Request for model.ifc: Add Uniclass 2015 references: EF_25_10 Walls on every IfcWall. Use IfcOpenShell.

First a look at what the model holds.

```python
import ifcopenshell

model = ifcopenshell.open("model.ifc")
print(model.schema)
print("classifications:", [c.Name for c in model.by_type("IfcClassification")])
for ifc_class in ("IfcDoor", "IfcRoof", "IfcStair", "IfcWall", "IfcWindow"):
    print(ifc_class, len(model.by_type(ifc_class)))
```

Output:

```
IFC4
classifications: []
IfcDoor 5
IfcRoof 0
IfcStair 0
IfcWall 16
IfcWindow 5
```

```python
import ifcopenshell
import ifcopenshell.api.classification

model = ifcopenshell.open("model.ifc")

system = ifcopenshell.api.classification.add_classification(model, classification="Uniclass 2015")

codes = {
    "IfcWall": ("EF_25_10", "Walls"),
}
for ifc_class, (code, name) in codes.items():
    products = model.by_type(ifc_class)
    ifcopenshell.api.classification.add_reference(
        model, products=products, classification=system, identification=code, name=name
    )
    print(code, len(products))

model.write("model_rev.ifc")
```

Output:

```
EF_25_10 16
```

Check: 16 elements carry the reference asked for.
